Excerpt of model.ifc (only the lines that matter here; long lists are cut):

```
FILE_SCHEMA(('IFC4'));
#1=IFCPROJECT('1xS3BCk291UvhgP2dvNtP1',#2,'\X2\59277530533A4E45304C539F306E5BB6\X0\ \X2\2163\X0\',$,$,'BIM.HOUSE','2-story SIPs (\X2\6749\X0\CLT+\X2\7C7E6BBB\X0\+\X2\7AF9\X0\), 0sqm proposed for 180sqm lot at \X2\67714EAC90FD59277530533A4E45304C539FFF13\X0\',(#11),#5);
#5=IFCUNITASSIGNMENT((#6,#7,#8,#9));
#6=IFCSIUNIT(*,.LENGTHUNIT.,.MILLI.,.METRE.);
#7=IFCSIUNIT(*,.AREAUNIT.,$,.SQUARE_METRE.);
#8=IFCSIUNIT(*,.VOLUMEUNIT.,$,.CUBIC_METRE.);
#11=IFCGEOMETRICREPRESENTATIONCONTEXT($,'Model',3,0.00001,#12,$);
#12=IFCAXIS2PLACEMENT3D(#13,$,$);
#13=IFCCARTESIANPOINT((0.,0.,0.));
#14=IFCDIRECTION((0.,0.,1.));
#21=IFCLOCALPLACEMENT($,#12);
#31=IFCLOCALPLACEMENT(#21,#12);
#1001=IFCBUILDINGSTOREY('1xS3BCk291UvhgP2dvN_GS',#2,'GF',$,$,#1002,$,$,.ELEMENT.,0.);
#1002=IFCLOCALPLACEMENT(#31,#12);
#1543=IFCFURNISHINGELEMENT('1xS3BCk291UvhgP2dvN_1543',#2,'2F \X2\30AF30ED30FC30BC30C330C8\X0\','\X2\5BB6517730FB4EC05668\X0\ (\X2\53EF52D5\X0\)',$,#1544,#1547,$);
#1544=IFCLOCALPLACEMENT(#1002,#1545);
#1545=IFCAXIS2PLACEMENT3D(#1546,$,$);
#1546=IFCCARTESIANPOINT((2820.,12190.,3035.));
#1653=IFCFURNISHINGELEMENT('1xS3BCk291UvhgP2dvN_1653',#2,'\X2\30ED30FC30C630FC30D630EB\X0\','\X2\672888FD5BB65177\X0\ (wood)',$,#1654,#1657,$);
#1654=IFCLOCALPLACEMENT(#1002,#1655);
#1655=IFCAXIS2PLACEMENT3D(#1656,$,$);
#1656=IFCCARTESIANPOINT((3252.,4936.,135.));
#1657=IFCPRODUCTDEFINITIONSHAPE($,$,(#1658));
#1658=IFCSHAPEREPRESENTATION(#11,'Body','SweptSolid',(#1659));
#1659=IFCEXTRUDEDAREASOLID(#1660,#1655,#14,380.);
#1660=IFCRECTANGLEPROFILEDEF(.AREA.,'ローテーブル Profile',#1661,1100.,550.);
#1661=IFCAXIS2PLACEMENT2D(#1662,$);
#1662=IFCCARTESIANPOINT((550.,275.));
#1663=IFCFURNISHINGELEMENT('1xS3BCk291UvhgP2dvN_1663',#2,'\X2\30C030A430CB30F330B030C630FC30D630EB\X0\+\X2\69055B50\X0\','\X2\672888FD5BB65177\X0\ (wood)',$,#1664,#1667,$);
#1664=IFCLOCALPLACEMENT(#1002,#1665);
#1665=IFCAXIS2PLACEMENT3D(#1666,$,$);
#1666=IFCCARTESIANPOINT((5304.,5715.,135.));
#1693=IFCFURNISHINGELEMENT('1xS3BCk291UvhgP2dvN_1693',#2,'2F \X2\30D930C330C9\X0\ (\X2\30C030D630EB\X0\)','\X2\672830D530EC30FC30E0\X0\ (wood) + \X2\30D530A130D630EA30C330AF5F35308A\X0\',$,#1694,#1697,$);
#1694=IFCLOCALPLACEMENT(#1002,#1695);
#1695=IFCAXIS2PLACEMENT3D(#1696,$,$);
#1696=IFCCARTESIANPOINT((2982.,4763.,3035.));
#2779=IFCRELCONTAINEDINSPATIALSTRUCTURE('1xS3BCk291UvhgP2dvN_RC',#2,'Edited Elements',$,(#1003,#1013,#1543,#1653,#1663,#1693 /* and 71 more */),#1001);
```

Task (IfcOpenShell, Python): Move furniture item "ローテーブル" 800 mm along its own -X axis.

```python
import ifcopenshell
import ifcopenshell.api.geometry
import ifcopenshell.util.placement
import ifcopenshell.util.unit

model = ifcopenshell.open("model.ifc")
unit_scale = ifcopenshell.util.unit.calculate_unit_scale(model)

item = model.by_guid("1xS3BCk291UvhgP2dvN_1653")
matrix = ifcopenshell.util.placement.get_local_placement(item.ObjectPlacement)
matrix[:3, 3] -= matrix[:3, 0] * 0.8 / unit_scale
ifcopenshell.api.geometry.edit_object_placement(model, product=item, matrix=matrix, is_si=False)

print(ifcopenshell.util.placement.get_local_placement(item.ObjectPlacement).round(3) + 0.0)

model.write("model-out.ifc")
```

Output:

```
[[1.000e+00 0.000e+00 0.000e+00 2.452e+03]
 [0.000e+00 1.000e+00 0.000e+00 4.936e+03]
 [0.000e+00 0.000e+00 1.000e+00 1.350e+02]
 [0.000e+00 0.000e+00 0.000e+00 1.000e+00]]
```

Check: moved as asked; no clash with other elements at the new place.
